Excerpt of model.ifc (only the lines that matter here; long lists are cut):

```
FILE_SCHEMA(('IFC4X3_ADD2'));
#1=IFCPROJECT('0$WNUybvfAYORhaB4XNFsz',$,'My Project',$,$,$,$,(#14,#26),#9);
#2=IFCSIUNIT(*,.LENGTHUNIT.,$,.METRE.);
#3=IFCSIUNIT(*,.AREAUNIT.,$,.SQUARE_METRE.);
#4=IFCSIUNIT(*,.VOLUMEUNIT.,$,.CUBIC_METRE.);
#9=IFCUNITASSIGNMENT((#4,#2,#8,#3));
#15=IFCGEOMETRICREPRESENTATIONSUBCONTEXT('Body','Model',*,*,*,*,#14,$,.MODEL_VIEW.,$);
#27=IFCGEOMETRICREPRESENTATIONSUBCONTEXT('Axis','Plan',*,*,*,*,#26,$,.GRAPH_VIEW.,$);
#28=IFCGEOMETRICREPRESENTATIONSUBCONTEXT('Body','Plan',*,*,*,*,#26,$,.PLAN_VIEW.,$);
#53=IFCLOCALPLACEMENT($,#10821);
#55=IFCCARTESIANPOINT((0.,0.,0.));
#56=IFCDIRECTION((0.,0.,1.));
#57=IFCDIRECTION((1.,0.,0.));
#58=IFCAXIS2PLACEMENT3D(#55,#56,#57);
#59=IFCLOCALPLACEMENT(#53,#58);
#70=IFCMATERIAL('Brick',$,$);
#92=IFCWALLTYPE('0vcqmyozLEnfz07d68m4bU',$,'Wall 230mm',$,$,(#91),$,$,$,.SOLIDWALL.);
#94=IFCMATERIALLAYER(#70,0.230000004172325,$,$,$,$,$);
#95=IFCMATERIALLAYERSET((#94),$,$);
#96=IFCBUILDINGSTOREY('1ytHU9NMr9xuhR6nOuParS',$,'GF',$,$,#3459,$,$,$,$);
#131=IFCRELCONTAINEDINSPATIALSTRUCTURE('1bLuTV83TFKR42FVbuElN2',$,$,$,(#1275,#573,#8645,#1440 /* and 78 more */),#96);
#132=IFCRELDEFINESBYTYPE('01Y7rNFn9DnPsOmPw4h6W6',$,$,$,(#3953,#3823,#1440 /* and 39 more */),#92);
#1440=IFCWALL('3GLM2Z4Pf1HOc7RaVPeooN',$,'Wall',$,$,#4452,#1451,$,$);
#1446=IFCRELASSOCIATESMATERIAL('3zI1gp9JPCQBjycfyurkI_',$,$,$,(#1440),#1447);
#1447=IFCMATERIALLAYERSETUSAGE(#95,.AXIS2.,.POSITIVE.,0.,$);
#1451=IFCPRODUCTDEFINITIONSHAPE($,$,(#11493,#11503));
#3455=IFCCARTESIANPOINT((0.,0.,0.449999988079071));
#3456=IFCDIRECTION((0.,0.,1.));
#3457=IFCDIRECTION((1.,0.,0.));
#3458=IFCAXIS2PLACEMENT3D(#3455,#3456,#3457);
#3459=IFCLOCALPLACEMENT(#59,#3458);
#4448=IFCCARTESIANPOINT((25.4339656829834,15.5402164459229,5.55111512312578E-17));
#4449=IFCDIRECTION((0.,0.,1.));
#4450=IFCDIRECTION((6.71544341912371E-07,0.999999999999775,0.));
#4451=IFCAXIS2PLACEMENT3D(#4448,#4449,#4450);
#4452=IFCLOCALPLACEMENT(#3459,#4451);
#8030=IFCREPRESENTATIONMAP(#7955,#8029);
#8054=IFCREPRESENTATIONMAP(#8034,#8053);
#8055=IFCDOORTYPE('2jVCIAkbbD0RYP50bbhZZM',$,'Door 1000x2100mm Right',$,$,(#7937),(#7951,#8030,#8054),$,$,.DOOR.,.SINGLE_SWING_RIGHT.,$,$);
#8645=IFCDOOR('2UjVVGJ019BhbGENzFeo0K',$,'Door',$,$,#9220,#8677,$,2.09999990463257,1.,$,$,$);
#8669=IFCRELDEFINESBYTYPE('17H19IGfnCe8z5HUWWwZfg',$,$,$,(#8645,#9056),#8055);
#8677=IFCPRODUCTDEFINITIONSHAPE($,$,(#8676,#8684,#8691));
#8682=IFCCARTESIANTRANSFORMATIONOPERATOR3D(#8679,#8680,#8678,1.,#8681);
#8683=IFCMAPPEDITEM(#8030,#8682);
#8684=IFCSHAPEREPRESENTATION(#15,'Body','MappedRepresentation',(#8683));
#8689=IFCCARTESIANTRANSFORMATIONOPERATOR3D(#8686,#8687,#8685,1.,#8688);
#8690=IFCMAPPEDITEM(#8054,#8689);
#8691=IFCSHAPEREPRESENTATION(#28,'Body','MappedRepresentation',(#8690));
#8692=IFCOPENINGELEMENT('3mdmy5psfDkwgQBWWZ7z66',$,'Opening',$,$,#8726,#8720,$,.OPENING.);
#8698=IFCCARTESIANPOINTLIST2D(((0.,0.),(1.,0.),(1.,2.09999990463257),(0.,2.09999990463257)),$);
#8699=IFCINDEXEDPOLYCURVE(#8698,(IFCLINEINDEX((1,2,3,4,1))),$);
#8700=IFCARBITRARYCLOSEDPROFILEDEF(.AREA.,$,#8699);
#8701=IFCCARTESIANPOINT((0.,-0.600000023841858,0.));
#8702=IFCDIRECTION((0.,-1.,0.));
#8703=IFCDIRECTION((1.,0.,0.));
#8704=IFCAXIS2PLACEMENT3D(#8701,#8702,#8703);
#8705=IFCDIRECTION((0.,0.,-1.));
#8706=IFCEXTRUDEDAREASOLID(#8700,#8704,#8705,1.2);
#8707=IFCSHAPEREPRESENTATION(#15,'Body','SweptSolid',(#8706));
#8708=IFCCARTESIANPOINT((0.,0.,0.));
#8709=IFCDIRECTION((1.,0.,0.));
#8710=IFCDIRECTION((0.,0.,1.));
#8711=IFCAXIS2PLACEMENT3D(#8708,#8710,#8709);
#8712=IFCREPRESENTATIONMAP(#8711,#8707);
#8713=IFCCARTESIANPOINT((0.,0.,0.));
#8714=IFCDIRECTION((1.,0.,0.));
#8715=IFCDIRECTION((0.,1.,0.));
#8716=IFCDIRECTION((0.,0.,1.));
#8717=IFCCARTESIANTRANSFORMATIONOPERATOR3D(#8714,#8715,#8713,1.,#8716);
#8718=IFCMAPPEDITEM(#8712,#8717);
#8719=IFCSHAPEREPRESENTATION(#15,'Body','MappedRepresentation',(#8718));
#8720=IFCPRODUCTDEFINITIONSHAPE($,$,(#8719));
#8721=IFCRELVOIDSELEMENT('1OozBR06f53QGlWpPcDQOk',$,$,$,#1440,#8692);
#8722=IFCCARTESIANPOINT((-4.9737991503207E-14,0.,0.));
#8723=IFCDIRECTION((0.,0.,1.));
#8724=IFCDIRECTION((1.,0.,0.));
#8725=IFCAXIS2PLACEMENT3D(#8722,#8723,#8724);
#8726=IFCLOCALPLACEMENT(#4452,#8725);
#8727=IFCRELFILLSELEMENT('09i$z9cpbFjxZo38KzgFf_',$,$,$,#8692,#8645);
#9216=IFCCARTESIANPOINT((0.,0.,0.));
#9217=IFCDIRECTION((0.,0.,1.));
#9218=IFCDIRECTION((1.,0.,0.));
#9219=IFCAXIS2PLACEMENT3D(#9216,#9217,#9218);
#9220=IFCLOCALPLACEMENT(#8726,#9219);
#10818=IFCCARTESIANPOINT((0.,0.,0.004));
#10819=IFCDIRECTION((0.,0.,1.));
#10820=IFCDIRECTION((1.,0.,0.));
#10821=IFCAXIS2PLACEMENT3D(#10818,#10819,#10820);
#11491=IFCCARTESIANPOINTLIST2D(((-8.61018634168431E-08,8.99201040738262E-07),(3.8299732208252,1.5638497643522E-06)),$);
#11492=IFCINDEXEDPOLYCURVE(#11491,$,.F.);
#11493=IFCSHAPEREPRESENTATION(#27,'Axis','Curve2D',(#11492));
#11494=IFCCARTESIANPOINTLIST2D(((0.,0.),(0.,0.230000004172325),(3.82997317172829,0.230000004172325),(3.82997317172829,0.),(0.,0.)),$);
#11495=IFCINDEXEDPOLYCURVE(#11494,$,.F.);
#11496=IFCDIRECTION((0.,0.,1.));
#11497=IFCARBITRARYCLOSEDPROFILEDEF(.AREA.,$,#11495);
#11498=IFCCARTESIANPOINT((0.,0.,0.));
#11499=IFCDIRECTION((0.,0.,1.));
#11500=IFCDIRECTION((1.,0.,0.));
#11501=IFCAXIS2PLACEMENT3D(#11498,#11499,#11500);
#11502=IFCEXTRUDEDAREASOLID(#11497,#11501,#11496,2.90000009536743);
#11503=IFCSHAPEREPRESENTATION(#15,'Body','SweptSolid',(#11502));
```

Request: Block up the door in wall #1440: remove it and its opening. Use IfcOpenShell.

```python
import ifcopenshell
import ifcopenshell.api.feature
import ifcopenshell.api.root
import ifcopenshell.geom
import ifcopenshell.util.shape

model = ifcopenshell.open("model.ifc")
settings = ifcopenshell.geom.settings()


def volume(element):
    """Net volume in cubic metres, openings subtracted."""
    shape = ifcopenshell.geom.create_shape(settings, element)
    return ifcopenshell.util.shape.get_volume(shape.geometry)


door = model.by_id(8645)
opening = door.FillsVoids[0].RelatingOpeningElement
wall = opening.VoidsElements[0].RelatingBuildingElement
before = volume(wall)

ifcopenshell.api.root.remove_product(model, product=door)
ifcopenshell.api.feature.remove_feature(model, feature=opening)

after = volume(wall)

print(f"wall volume {before:.3f} -> {after:.3f} m3")

model.write("model_v2.ifc")
```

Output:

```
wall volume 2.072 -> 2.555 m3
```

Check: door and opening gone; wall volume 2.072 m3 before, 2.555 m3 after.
